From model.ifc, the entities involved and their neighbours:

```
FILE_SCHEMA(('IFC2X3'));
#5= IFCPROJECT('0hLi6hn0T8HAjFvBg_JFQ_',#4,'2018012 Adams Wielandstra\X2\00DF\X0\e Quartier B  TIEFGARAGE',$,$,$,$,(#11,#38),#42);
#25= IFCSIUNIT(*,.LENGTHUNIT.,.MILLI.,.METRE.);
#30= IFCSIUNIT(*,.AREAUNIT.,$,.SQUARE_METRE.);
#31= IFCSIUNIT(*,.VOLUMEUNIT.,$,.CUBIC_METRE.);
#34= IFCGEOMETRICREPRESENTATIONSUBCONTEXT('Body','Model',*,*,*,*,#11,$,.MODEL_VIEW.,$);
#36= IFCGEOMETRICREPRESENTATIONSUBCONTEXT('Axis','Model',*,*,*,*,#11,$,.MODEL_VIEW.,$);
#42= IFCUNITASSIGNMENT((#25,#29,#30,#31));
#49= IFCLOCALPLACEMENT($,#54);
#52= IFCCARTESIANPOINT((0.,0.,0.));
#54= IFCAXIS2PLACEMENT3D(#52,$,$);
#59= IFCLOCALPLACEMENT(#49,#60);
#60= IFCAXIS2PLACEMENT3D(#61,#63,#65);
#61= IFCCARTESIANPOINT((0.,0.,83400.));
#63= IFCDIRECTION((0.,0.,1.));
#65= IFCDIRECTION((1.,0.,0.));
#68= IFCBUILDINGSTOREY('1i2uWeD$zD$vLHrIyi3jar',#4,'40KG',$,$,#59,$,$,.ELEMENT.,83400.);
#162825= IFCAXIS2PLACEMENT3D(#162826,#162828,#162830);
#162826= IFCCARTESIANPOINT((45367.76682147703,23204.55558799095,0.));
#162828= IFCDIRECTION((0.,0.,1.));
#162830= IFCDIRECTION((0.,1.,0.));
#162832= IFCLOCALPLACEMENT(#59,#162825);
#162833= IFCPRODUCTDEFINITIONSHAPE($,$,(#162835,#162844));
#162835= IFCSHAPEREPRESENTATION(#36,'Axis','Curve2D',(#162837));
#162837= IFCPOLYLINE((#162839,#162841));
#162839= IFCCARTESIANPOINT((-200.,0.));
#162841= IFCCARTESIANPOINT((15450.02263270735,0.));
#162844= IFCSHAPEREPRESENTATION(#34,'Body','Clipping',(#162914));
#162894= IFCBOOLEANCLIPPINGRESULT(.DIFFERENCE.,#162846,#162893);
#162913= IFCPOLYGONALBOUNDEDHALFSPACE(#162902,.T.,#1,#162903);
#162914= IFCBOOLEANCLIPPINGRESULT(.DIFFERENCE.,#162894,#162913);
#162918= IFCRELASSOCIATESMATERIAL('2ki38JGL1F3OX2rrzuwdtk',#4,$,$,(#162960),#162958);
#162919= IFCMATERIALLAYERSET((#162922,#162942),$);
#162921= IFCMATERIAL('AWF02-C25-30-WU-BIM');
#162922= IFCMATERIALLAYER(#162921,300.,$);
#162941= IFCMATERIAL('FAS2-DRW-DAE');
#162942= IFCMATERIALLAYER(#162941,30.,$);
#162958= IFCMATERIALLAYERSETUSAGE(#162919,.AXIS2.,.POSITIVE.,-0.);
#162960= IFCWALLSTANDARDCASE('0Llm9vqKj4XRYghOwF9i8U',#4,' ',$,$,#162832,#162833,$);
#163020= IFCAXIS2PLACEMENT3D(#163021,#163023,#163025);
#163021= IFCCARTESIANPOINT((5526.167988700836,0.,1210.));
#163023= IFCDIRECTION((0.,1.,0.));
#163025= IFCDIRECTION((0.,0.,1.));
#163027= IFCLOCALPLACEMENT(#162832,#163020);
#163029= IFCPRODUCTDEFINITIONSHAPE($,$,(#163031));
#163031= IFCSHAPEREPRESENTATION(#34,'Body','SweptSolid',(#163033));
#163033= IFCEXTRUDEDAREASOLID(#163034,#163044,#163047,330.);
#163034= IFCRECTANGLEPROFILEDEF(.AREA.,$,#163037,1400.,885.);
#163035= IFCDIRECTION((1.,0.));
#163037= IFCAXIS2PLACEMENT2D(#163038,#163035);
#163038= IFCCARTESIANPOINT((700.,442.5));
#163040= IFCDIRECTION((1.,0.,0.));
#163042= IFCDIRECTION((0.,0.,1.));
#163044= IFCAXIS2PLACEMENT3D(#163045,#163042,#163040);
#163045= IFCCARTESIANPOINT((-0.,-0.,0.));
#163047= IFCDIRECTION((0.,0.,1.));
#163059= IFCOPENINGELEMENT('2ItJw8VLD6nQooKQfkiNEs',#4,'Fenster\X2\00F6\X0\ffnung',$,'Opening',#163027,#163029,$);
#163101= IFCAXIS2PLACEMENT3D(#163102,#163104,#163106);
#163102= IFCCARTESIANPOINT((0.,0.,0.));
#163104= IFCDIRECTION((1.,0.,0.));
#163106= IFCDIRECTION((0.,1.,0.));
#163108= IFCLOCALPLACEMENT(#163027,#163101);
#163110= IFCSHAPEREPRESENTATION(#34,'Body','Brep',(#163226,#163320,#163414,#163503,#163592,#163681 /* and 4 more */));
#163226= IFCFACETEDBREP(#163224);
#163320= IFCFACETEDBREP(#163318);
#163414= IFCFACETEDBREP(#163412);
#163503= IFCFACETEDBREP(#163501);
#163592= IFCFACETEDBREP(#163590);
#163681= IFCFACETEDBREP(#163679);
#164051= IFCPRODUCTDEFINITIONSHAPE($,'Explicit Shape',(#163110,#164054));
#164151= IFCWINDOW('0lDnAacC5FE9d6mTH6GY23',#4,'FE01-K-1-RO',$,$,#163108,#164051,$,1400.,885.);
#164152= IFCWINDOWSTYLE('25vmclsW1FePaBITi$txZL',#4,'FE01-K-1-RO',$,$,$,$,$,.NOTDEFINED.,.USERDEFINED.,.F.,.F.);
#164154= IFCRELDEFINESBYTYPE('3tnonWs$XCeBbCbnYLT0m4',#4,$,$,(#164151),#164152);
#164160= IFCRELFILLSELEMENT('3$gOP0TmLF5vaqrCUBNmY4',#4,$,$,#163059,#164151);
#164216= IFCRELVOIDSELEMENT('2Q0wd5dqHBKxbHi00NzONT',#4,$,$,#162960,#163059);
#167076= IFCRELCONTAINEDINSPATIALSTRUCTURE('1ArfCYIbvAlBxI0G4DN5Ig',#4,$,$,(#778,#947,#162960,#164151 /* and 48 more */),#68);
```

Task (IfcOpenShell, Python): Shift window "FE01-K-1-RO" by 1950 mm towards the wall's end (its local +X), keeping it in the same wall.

```python
import ifcopenshell
import ifcopenshell.api.geometry
import ifcopenshell.util.placement

model = ifcopenshell.open("model.ifc")

window = model.by_guid("0lDnAacC5FE9d6mTH6GY23")
opening = window.FillsVoids[0].RelatingOpeningElement
wall = opening.VoidsElements[0].RelatingBuildingElement

wall_matrix = ifcopenshell.util.placement.get_local_placement(wall.ObjectPlacement)
shift = wall_matrix[:3, 0] * 1950.0
before = ifcopenshell.util.placement.get_local_placement(window.ObjectPlacement)[:3, 3].copy()

# The window is placed relative to its opening, so it follows when the opening moves.
matrix = ifcopenshell.util.placement.get_local_placement(opening.ObjectPlacement)
matrix[:3, 3] += shift
ifcopenshell.api.geometry.edit_object_placement(
    model, product=opening, matrix=matrix, is_si=False, should_transform_children=True
)

after = ifcopenshell.util.placement.get_local_placement(window.ObjectPlacement)[:3, 3]
print("window moved by", (after - before).round(3) + 0.0)

model.write("model_updated.ifc")
```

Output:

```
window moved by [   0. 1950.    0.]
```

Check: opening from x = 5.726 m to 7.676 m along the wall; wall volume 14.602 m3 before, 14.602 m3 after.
